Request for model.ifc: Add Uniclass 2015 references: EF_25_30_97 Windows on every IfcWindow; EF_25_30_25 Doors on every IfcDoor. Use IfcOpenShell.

First a look at what the model holds.

```python
import ifcopenshell

model = ifcopenshell.open("model.ifc")
print(model.schema)
print("classifications:", [c.Name for c in model.by_type("IfcClassification")])
for ifc_class in ("IfcDoor", "IfcRoof", "IfcStair", "IfcWall", "IfcWindow"):
    print(ifc_class, len(model.by_type(ifc_class)))
```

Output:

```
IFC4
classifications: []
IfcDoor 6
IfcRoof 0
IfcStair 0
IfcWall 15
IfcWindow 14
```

```python
import ifcopenshell
import ifcopenshell.api.classification

model = ifcopenshell.open("model.ifc")

system = ifcopenshell.api.classification.add_classification(model, classification="Uniclass 2015")

codes = {
    "IfcWindow": ("EF_25_30_97", "Windows"),
    "IfcDoor": ("EF_25_30_25", "Doors"),
}
for ifc_class, (code, name) in codes.items():
    products = model.by_type(ifc_class)
    ifcopenshell.api.classification.add_reference(
        model, products=products, classification=system, identification=code, name=name
    )
    print(code, len(products))

model.write("model_rev.ifc")
```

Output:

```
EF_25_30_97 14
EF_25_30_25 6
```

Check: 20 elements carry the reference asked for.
